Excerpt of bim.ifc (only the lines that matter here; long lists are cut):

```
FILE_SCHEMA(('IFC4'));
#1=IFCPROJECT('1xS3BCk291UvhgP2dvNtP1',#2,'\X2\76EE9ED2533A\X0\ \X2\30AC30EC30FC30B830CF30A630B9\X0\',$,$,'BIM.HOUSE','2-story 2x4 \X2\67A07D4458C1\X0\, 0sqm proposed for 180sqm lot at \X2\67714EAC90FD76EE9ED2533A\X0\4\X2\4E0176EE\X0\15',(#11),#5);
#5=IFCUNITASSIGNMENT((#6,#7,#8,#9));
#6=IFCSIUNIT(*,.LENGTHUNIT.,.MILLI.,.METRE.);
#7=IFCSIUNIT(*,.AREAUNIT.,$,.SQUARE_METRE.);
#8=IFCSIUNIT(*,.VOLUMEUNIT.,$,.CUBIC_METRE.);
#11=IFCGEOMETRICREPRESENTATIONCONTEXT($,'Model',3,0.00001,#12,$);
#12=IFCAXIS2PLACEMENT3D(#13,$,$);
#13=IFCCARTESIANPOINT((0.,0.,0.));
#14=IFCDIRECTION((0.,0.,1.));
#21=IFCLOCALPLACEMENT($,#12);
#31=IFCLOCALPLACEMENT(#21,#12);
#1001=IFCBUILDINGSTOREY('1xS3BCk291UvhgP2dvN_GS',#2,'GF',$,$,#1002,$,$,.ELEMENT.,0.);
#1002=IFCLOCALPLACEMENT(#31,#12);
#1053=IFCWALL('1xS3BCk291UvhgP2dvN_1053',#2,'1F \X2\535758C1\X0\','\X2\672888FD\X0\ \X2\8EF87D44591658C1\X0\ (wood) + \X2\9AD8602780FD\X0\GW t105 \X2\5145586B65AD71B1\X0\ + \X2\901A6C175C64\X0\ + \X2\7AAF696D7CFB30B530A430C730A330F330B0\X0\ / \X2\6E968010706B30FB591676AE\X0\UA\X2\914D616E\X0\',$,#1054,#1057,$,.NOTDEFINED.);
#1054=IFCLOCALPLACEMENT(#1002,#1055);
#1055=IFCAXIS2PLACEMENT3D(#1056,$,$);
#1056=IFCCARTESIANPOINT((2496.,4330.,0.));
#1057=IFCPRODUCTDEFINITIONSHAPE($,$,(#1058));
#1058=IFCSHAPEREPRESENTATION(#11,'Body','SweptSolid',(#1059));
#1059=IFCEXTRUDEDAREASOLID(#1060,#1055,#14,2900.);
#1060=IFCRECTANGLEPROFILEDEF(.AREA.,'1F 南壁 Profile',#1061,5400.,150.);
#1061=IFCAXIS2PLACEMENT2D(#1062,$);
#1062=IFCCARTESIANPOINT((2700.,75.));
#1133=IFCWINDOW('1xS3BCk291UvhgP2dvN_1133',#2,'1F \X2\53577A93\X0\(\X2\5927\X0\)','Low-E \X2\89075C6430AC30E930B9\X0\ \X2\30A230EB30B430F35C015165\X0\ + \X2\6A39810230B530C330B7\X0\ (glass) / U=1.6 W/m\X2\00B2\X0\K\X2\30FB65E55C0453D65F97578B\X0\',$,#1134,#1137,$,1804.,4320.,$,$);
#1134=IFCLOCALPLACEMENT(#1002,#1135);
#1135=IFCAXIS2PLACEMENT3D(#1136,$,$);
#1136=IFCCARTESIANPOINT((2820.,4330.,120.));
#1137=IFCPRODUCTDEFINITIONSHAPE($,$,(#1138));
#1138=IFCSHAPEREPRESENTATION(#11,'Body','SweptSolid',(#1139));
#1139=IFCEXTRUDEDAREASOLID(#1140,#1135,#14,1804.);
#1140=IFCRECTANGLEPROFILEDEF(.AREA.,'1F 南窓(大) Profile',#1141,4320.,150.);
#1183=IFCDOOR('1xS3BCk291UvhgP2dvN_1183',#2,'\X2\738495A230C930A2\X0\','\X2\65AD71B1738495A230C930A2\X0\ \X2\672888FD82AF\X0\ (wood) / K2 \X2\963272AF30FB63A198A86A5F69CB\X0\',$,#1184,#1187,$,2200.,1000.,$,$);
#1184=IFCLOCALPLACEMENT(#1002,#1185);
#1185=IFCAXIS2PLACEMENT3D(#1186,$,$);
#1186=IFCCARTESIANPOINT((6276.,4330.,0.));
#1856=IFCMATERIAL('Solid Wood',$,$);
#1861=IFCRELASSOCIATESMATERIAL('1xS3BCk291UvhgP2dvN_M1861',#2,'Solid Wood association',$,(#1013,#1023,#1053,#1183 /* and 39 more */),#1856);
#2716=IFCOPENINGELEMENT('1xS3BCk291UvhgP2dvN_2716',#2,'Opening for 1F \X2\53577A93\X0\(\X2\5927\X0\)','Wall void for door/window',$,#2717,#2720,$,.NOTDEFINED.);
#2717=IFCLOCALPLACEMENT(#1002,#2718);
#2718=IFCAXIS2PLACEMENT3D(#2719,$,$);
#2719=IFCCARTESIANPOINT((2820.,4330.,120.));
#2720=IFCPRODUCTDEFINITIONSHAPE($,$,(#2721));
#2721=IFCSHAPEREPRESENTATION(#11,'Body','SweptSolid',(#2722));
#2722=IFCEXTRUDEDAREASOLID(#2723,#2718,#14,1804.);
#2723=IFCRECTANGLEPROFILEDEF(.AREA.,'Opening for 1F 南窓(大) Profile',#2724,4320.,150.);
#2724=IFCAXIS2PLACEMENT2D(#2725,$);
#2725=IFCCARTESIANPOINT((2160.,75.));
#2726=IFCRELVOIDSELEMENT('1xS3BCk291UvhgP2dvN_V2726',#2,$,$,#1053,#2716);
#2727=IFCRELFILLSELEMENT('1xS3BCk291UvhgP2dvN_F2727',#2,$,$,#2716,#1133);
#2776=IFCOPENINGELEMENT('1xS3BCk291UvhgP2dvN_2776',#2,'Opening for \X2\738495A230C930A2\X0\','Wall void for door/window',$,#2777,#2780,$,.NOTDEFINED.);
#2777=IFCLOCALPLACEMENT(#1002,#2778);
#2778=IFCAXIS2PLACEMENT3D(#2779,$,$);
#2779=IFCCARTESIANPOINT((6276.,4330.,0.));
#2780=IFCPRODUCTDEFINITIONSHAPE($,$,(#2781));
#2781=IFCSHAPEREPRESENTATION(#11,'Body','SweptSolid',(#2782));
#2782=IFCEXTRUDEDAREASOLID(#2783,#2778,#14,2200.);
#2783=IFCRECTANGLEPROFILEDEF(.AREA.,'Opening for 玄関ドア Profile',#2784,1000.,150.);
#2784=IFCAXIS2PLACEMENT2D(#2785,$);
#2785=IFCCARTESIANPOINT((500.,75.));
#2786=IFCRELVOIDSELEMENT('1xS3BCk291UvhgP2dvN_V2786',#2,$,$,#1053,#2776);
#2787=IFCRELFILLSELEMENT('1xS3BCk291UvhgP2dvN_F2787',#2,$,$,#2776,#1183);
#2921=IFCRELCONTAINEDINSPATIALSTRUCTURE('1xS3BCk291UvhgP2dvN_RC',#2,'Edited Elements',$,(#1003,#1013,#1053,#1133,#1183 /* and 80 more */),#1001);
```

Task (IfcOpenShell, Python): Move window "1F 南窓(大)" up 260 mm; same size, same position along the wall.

```python
import numpy as np
import ifcopenshell
import ifcopenshell.api.geometry
import ifcopenshell.util.placement
import ifcopenshell.util.unit

model = ifcopenshell.open("bim.ifc")
unit_scale = ifcopenshell.util.unit.calculate_unit_scale(model)

window = model.by_guid("1xS3BCk291UvhgP2dvN_1133")
opening = window.FillsVoids[0].RelatingOpeningElement
dz = 260.0

shift = np.array([0.0, 0.0, dz])
# The window is not placed relative to its opening, so move both.
for product in (opening, window):
    matrix = ifcopenshell.util.placement.get_local_placement(product.ObjectPlacement)
    matrix[:3, 3] += shift
    ifcopenshell.api.geometry.edit_object_placement(model, product=product, matrix=matrix, is_si=False)

print(f"moved by {dz * unit_scale:+.3f} m")

model.write("bim_rev.ifc")
```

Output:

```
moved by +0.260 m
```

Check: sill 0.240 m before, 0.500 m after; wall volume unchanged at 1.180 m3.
